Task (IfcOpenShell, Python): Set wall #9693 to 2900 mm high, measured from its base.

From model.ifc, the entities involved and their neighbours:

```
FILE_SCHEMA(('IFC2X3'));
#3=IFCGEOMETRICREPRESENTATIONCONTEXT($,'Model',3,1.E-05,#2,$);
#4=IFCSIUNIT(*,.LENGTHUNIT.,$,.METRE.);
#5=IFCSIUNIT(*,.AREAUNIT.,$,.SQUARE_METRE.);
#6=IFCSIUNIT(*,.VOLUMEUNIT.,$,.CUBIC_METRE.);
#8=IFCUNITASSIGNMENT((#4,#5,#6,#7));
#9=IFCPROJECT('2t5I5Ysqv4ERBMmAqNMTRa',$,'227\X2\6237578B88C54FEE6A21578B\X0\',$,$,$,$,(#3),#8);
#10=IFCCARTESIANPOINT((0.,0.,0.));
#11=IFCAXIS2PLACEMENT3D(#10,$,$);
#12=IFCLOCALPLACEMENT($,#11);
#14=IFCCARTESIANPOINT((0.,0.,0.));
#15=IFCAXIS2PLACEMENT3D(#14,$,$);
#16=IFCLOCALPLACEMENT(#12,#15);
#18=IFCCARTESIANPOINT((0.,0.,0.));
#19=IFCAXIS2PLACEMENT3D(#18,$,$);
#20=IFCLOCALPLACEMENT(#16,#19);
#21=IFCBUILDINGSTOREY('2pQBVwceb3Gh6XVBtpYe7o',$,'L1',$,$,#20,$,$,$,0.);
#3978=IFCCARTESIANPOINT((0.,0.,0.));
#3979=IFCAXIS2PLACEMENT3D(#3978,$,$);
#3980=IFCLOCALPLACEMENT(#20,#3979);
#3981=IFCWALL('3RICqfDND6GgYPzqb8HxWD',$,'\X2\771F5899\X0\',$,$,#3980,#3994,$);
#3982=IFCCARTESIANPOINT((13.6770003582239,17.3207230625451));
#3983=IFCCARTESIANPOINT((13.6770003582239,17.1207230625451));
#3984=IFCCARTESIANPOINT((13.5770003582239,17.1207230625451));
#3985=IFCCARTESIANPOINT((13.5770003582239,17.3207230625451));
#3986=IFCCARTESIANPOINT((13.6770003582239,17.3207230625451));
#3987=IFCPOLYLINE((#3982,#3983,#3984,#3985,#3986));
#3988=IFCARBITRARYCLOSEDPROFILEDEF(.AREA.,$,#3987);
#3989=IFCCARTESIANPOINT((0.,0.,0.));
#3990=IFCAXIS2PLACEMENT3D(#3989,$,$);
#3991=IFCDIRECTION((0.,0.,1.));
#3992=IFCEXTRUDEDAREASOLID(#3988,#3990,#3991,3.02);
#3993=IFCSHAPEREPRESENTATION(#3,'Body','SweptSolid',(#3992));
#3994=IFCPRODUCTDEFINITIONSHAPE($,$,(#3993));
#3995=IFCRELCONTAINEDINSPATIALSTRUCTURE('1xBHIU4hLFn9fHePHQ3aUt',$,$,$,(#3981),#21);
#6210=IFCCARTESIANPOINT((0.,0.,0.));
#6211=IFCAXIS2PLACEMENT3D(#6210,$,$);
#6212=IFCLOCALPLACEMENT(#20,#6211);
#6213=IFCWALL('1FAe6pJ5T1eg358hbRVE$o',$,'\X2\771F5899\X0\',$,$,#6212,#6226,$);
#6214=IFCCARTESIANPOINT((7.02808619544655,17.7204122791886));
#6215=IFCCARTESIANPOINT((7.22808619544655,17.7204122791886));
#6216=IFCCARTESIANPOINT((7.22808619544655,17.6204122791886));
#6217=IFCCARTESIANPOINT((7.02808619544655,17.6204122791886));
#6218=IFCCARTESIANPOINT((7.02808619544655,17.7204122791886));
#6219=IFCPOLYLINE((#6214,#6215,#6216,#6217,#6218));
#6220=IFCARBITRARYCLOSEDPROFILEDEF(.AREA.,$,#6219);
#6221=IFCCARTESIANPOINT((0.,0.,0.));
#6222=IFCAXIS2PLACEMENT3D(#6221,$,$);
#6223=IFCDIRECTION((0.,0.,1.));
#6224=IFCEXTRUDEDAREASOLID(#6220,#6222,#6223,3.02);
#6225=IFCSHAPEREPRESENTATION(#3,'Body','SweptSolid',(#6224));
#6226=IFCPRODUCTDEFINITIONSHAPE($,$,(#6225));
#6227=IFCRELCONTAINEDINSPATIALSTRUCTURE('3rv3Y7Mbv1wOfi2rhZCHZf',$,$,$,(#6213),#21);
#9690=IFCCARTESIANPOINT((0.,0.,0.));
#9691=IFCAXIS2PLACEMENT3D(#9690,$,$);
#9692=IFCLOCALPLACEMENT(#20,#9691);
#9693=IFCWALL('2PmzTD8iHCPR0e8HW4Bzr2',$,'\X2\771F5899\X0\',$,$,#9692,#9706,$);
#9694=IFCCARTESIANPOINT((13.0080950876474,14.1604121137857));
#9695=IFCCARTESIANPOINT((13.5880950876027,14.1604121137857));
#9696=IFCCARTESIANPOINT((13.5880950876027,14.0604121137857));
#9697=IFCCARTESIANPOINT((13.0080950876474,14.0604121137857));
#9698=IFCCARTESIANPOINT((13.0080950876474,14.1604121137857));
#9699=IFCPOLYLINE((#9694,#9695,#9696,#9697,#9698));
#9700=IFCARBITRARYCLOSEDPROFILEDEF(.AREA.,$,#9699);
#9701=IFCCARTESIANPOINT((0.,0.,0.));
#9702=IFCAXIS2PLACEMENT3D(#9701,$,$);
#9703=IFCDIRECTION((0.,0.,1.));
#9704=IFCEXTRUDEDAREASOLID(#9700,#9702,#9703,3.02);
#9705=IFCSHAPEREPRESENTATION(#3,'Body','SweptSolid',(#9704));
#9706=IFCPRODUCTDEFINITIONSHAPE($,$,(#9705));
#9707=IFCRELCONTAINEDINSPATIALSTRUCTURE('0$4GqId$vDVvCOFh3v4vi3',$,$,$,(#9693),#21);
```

```python
import ifcopenshell
import ifcopenshell.geom
import ifcopenshell.util.shape
import ifcopenshell.util.unit

model = ifcopenshell.open("model.ifc")
unit_scale = ifcopenshell.util.unit.calculate_unit_scale(model)
settings = ifcopenshell.geom.settings()


def volume(element):
    """Net volume in cubic metres, openings subtracted."""
    shape = ifcopenshell.geom.create_shape(settings, element)
    return ifcopenshell.util.shape.get_volume(shape.geometry)


wall = model.by_guid("2PmzTD8iHCPR0e8HW4Bzr2")
before = volume(wall)

body = next(r for r in wall.Representation.Representations if r.RepresentationIdentifier == "Body")
solid = body.Items[0]
old_height = solid.Depth
solid.Depth = 2.9 / unit_scale
after = volume(wall)

print(f"height {old_height:g} -> {solid.Depth:g}, volume {before:.3f} -> {after:.3f} m3")

model.write("model-out.ifc")
```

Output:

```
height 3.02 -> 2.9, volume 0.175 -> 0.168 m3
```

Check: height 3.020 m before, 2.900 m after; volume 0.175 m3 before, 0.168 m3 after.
